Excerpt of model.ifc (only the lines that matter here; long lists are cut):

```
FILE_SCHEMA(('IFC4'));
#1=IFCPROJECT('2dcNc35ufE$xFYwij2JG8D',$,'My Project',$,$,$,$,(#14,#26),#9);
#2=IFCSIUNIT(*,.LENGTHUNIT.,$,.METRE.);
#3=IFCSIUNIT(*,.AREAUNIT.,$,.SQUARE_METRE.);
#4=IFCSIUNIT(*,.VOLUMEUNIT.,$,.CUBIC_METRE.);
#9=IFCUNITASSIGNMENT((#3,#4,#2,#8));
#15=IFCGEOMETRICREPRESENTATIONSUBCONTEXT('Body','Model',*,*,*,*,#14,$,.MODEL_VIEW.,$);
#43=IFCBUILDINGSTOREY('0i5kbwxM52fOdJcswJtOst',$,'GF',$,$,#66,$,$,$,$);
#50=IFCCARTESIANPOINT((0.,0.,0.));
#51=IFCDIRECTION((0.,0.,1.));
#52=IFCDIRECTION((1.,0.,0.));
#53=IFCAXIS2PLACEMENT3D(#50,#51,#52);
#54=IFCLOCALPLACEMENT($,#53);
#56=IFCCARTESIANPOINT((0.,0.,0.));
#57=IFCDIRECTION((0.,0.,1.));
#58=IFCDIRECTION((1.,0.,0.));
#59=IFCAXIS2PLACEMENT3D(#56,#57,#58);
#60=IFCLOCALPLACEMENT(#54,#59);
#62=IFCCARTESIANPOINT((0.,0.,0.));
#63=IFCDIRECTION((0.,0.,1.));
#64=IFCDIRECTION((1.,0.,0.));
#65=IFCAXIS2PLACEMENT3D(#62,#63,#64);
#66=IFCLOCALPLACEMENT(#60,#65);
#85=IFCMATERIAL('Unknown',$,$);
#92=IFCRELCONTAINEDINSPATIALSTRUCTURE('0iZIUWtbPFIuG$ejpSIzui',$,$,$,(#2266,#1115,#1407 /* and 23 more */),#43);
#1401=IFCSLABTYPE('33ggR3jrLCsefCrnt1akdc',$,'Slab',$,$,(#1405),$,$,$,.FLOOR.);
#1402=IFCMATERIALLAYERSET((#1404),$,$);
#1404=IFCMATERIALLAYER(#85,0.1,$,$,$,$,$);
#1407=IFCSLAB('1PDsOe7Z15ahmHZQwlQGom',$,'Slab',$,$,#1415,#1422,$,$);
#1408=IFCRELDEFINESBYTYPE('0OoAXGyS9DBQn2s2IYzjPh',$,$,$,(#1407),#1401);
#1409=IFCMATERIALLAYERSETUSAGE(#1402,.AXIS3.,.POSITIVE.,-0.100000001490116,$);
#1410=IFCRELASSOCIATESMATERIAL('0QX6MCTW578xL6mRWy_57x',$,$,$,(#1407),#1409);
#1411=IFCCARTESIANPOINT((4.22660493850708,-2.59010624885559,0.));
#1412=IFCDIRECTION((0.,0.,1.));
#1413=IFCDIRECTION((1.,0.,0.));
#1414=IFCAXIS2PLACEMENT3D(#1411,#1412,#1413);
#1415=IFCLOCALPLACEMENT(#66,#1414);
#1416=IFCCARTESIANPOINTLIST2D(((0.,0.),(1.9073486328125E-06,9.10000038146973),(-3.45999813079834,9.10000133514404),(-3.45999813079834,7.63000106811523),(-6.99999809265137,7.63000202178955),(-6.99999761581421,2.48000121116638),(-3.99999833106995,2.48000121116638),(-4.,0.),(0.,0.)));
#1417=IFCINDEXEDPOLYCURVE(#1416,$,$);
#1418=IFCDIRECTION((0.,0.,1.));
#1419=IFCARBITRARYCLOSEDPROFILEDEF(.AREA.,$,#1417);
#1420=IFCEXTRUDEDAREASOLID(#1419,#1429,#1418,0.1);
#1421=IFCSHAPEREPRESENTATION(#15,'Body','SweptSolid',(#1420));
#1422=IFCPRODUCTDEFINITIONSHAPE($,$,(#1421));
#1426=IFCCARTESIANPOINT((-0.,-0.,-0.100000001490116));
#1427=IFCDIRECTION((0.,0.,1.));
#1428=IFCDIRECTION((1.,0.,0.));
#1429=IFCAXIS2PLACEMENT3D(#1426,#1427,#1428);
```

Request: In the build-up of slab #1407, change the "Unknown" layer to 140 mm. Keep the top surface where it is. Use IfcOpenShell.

```python
import ifcopenshell
import ifcopenshell.util.element
import ifcopenshell.util.representation

model = ifcopenshell.open("model.ifc")

layer_set = model.by_id(1402)
layer = next(l for l in layer_set.MaterialLayers if l.Material and l.Material.Name == "Unknown")
change = 0.14 - layer.LayerThickness
layer.LayerThickness += change

# Geometry does not follow the layer set by itself.
slabs = [e for e in ifcopenshell.util.element.get_elements_by_material(model, layer_set) if e.is_a("IfcSlab")]
for slab in sorted(slabs, key=lambda e: e.id()):
    body = ifcopenshell.util.representation.get_representation(slab, "Model", "Body")
    solid = body.Items[0]
    old_depth = solid.Depth
    solid.Depth += change
    # Extruded upwards: lower the start of the extrusion so the top stays.
    x, y, z = solid.Position.Location.Coordinates
    solid.Position.Location = model.createIfcCartesianPoint((x, y, z - change))
    print(slab.id(), f"{old_depth:g} -> {solid.Depth:g}")

# The layers are counted up from the underside, which has moved.
for usage in {ifcopenshell.util.element.get_material(slab) for slab in slabs}:
    usage.OffsetFromReferenceLine -= change

model.write("model_v2.ifc")
```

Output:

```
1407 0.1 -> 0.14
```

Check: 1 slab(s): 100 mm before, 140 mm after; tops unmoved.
